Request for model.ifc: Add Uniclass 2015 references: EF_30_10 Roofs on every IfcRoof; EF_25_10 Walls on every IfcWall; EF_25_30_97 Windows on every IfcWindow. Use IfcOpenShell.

First a look at what the model holds.

```python
import ifcopenshell

model = ifcopenshell.open("model.ifc")
print(model.schema)
print("classifications:", [c.Name for c in model.by_type("IfcClassification")])
for ifc_class in ("IfcDoor", "IfcRoof", "IfcStair", "IfcWall", "IfcWindow"):
    print(ifc_class, len(model.by_type(ifc_class)))
```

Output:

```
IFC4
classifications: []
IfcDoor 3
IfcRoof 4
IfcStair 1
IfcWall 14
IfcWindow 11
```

```python
import ifcopenshell
import ifcopenshell.api.classification

model = ifcopenshell.open("model.ifc")

system = ifcopenshell.api.classification.add_classification(model, classification="Uniclass 2015")

codes = {
    "IfcRoof": ("EF_30_10", "Roofs"),
    "IfcWall": ("EF_25_10", "Walls"),
    "IfcWindow": ("EF_25_30_97", "Windows"),
}
for ifc_class, (code, name) in codes.items():
    products = model.by_type(ifc_class)
    ifcopenshell.api.classification.add_reference(
        model, products=products, classification=system, identification=code, name=name
    )
    print(code, len(products))

model.write("model_v2.ifc")
```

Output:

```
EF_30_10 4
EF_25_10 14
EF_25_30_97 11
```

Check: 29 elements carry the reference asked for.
